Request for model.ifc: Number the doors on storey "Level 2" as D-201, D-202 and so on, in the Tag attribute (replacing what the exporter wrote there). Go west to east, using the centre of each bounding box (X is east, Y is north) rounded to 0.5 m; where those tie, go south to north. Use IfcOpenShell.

First a look at what the model holds.

```python
import ifcopenshell
import ifcopenshell.util.element
import ifcopenshell.util.placement

model = ifcopenshell.open("model.ifc")
print(model.schema)
storey = next(s for s in model.by_type("IfcBuildingStorey") if s.Name == "Level 2")
doors = [e for e in ifcopenshell.util.element.get_decomposition(storey) if e.is_a("IfcDoor")]
for e in sorted(doors, key=lambda e: e.id()):
    origin = ifcopenshell.util.placement.get_local_placement(e.ObjectPlacement)[:3, 3]
    print(e.id(), e.Tag, e.Name, origin.round(2) + 0.0, sep=" | ")
```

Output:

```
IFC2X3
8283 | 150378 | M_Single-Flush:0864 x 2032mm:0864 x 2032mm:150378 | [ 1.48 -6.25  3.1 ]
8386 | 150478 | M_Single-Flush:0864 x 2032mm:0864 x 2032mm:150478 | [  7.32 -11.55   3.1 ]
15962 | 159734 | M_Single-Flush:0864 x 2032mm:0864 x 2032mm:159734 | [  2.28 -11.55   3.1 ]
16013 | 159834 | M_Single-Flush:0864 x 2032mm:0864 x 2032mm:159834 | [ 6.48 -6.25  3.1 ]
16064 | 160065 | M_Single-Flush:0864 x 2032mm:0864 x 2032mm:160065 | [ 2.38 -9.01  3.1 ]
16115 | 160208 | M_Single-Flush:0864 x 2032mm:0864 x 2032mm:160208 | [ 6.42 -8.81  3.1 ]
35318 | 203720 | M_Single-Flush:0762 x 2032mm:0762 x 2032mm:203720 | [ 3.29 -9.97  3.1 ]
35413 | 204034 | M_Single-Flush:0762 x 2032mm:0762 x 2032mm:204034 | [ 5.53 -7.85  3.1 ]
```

```python
import ifcopenshell
import ifcopenshell.geom
import ifcopenshell.util.element
import ifcopenshell.util.shape

model = ifcopenshell.open("model.ifc")
settings = ifcopenshell.geom.settings()
settings.set("use-world-coords", True)


def centre(element):
    shape = ifcopenshell.geom.create_shape(settings, element)
    return ifcopenshell.util.shape.get_bbox_centroid(shape.geometry)


storey = next(s for s in model.by_type("IfcBuildingStorey") if s.Name == "Level 2")
doors = [e for e in ifcopenshell.util.element.get_decomposition(storey) if e.is_a("IfcDoor")]

# Insertion points can sit at a corner or the storey origin, so sort by the geometry (in metres).
centres = {e: centre(e) for e in doors}
doors.sort(key=lambda e: (round(centres[e][0] / 0.5), centres[e][1]))

for i, e in enumerate(doors, start=1):
    number = f"D-2{i:02d}"
    e.Tag = number
    print(e.id(), number)

model.write("model_updated.ifc")
```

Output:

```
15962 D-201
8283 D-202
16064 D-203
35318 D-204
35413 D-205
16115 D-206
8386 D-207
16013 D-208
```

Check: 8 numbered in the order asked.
